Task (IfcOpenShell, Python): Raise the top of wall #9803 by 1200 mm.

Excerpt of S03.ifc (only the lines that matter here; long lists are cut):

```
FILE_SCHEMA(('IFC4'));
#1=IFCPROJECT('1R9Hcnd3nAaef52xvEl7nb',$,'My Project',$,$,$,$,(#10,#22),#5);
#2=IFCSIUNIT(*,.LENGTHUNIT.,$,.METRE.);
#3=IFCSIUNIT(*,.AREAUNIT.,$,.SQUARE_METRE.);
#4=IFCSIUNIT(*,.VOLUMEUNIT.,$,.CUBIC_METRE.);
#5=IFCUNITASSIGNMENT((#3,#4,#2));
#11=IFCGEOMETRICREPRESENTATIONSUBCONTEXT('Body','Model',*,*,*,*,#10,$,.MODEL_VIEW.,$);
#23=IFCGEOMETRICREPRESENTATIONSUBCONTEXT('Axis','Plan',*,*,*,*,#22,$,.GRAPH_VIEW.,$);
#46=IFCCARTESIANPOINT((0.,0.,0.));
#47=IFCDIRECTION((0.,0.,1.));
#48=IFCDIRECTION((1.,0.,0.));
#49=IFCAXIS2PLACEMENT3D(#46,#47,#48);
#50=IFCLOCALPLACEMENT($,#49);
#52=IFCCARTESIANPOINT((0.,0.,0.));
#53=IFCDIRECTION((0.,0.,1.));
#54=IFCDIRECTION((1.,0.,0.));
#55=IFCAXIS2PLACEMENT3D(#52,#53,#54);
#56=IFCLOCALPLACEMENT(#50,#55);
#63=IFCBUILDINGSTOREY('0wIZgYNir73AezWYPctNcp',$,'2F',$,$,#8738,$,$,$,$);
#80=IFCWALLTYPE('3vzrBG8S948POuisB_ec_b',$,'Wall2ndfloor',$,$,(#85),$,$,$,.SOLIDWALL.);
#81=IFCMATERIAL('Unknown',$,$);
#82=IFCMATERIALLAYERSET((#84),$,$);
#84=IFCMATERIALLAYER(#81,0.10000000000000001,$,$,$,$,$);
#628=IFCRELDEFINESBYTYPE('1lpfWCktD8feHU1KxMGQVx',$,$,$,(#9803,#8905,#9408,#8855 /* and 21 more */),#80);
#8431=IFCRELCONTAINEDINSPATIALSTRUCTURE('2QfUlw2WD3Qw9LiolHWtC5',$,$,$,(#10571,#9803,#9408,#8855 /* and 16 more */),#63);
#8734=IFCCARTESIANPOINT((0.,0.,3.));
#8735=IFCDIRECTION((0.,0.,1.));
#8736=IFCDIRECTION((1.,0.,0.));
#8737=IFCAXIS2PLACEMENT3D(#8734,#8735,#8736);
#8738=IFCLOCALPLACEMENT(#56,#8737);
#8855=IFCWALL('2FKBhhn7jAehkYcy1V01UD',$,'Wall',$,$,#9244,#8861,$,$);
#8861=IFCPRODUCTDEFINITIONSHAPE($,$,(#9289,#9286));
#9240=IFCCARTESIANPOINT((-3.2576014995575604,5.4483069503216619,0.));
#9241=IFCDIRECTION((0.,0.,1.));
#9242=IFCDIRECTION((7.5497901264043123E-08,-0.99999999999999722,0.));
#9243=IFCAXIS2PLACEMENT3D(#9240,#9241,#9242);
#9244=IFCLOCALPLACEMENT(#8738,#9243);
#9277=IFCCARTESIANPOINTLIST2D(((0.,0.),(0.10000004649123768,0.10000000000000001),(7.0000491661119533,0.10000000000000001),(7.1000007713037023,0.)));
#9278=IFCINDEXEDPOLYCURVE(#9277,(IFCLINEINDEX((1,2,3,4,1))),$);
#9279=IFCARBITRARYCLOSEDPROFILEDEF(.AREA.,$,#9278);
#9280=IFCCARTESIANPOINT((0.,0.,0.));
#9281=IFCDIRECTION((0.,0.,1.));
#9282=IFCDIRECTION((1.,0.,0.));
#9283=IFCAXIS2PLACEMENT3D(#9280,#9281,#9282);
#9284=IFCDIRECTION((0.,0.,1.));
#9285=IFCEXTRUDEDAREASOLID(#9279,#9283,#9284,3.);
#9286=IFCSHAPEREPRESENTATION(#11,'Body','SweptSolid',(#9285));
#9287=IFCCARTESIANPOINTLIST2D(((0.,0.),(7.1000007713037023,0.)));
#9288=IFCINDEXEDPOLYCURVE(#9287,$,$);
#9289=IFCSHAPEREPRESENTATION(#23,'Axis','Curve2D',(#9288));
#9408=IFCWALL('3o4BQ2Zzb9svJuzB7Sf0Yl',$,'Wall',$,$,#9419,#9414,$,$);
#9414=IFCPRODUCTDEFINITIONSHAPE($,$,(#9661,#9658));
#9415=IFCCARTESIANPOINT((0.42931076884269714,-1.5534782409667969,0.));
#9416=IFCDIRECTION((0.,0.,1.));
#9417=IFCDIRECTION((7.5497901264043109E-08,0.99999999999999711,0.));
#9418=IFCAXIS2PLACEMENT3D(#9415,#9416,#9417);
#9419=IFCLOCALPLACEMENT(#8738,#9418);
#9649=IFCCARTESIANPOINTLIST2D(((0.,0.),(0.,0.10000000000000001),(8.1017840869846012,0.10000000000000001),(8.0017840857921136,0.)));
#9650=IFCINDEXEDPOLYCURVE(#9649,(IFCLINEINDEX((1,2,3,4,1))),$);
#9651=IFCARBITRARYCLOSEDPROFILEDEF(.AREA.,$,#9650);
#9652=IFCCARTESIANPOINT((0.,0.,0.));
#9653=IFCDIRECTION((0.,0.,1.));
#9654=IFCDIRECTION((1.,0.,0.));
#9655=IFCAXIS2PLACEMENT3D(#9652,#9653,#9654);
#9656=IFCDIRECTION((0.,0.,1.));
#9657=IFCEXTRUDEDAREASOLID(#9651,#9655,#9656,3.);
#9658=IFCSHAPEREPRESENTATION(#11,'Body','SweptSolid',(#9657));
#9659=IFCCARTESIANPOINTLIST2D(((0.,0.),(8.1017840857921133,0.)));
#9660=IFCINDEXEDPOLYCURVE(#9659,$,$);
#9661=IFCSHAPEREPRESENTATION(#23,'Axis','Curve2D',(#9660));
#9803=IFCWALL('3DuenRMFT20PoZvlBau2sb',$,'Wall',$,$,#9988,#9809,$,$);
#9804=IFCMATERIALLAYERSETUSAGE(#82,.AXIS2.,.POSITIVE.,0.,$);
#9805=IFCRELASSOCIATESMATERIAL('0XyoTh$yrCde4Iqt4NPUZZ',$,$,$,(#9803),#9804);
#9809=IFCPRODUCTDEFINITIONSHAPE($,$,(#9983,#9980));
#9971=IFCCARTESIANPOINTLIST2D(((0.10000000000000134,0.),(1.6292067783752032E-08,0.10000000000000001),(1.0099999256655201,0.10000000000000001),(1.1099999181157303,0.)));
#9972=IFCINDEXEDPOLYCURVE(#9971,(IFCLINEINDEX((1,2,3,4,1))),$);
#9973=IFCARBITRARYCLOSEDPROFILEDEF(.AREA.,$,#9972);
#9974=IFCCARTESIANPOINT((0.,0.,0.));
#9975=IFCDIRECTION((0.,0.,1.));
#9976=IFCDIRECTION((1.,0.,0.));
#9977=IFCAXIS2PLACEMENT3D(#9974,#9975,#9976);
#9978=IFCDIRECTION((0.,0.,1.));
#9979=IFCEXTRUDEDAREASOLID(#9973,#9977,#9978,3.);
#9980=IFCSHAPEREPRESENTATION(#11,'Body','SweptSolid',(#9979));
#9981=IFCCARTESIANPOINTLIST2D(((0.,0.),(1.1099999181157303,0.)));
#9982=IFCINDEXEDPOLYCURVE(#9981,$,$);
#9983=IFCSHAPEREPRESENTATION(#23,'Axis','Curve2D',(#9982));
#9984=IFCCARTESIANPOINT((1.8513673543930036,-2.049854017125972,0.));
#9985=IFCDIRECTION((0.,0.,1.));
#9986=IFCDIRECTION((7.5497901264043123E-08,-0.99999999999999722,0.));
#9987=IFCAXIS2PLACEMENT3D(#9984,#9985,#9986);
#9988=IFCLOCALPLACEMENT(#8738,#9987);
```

```python
import ifcopenshell
import ifcopenshell.geom
import ifcopenshell.util.representation
import ifcopenshell.util.shape
import ifcopenshell.util.unit

model = ifcopenshell.open("S03.ifc")
unit_scale = ifcopenshell.util.unit.calculate_unit_scale(model)
settings = ifcopenshell.geom.settings()


def volume(element):
    """Net volume in cubic metres, openings subtracted."""
    shape = ifcopenshell.geom.create_shape(settings, element)
    return ifcopenshell.util.shape.get_volume(shape.geometry)


wall = model.by_id(9803)
before = volume(wall)

body = ifcopenshell.util.representation.get_representation(wall, "Model", "Body")
solid = body.Items[0]
old_height = solid.Depth
solid.Depth += 1.2 / unit_scale
after = volume(wall)

print(f"height {old_height:g} -> {solid.Depth:g}, volume {before:.3f} -> {after:.3f} m3")

model.write("S03_v2.ifc")
```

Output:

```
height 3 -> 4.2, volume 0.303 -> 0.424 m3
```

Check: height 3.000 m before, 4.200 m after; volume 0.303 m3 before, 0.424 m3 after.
